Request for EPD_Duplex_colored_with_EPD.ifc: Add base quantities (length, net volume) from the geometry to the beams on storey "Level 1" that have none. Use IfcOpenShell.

First a look at what the model holds.

```python
import ifcopenshell
import ifcopenshell.util.element
import ifcopenshell.util.unit

model = ifcopenshell.open("EPD_Duplex_colored_with_EPD.ifc")
print(model.schema)
for unit_type in ("LENGTHUNIT", "AREAUNIT", "VOLUMEUNIT"):
    print(unit_type, ifcopenshell.util.unit.calculate_unit_scale(model, unit_type))
storey = next(s for s in model.by_type("IfcBuildingStorey") if s.Name == "Level 1")
beams = [e for e in ifcopenshell.util.element.get_decomposition(storey) if e.is_a("IfcBeam")]
for e in sorted(beams, key=lambda e: e.id()):
    print(e.id(), e.is_a(), e.Name, list(ifcopenshell.util.element.get_psets(e, qtos_only=True)), sep=" | ")
```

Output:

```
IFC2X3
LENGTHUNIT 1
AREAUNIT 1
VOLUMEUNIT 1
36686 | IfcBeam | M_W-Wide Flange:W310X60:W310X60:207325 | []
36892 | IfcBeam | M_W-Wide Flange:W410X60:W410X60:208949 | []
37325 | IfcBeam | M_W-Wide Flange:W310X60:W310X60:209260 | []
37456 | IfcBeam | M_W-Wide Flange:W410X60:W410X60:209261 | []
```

```python
import ifcopenshell
import ifcopenshell.api.pset
import ifcopenshell.geom
import ifcopenshell.util.element
import ifcopenshell.util.shape
import ifcopenshell.util.unit

model = ifcopenshell.open("EPD_Duplex_colored_with_EPD.ifc")
unit_scale = ifcopenshell.util.unit.calculate_unit_scale(model)
volume_scale = ifcopenshell.util.unit.calculate_unit_scale(model, "VOLUMEUNIT")
settings = ifcopenshell.geom.settings()

storey = next(s for s in model.by_type("IfcBuildingStorey") if s.Name == "Level 1")
beams = [e for e in ifcopenshell.util.element.get_decomposition(storey) if e.is_a("IfcBeam")]

for e in sorted(beams, key=lambda e: e.id()):
    if ifcopenshell.util.element.get_psets(e, qtos_only=True, should_inherit=False):
        continue
    # Geometry comes back in metres, in the element's own axes.
    shape = ifcopenshell.geom.create_shape(settings, e)
    values = {
        "Length": ifcopenshell.util.shape.get_max_xyz(shape.geometry) / unit_scale,
        "NetVolume": ifcopenshell.util.shape.get_volume(shape.geometry) / volume_scale,
    }
    qto = ifcopenshell.api.pset.add_qto(model, product=e, name="BaseQuantities")
    ifcopenshell.api.pset.edit_qto(model, qto=qto, properties=values)
    print(e.id(), {k: round(v, 3) for k, v in values.items()})

model.write("EPD_Duplex_colored_with_EPD_rev.ifc")
```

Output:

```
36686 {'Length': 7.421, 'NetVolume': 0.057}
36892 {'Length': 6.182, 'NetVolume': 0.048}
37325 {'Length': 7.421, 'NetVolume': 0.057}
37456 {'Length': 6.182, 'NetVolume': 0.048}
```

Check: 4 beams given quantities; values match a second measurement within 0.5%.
